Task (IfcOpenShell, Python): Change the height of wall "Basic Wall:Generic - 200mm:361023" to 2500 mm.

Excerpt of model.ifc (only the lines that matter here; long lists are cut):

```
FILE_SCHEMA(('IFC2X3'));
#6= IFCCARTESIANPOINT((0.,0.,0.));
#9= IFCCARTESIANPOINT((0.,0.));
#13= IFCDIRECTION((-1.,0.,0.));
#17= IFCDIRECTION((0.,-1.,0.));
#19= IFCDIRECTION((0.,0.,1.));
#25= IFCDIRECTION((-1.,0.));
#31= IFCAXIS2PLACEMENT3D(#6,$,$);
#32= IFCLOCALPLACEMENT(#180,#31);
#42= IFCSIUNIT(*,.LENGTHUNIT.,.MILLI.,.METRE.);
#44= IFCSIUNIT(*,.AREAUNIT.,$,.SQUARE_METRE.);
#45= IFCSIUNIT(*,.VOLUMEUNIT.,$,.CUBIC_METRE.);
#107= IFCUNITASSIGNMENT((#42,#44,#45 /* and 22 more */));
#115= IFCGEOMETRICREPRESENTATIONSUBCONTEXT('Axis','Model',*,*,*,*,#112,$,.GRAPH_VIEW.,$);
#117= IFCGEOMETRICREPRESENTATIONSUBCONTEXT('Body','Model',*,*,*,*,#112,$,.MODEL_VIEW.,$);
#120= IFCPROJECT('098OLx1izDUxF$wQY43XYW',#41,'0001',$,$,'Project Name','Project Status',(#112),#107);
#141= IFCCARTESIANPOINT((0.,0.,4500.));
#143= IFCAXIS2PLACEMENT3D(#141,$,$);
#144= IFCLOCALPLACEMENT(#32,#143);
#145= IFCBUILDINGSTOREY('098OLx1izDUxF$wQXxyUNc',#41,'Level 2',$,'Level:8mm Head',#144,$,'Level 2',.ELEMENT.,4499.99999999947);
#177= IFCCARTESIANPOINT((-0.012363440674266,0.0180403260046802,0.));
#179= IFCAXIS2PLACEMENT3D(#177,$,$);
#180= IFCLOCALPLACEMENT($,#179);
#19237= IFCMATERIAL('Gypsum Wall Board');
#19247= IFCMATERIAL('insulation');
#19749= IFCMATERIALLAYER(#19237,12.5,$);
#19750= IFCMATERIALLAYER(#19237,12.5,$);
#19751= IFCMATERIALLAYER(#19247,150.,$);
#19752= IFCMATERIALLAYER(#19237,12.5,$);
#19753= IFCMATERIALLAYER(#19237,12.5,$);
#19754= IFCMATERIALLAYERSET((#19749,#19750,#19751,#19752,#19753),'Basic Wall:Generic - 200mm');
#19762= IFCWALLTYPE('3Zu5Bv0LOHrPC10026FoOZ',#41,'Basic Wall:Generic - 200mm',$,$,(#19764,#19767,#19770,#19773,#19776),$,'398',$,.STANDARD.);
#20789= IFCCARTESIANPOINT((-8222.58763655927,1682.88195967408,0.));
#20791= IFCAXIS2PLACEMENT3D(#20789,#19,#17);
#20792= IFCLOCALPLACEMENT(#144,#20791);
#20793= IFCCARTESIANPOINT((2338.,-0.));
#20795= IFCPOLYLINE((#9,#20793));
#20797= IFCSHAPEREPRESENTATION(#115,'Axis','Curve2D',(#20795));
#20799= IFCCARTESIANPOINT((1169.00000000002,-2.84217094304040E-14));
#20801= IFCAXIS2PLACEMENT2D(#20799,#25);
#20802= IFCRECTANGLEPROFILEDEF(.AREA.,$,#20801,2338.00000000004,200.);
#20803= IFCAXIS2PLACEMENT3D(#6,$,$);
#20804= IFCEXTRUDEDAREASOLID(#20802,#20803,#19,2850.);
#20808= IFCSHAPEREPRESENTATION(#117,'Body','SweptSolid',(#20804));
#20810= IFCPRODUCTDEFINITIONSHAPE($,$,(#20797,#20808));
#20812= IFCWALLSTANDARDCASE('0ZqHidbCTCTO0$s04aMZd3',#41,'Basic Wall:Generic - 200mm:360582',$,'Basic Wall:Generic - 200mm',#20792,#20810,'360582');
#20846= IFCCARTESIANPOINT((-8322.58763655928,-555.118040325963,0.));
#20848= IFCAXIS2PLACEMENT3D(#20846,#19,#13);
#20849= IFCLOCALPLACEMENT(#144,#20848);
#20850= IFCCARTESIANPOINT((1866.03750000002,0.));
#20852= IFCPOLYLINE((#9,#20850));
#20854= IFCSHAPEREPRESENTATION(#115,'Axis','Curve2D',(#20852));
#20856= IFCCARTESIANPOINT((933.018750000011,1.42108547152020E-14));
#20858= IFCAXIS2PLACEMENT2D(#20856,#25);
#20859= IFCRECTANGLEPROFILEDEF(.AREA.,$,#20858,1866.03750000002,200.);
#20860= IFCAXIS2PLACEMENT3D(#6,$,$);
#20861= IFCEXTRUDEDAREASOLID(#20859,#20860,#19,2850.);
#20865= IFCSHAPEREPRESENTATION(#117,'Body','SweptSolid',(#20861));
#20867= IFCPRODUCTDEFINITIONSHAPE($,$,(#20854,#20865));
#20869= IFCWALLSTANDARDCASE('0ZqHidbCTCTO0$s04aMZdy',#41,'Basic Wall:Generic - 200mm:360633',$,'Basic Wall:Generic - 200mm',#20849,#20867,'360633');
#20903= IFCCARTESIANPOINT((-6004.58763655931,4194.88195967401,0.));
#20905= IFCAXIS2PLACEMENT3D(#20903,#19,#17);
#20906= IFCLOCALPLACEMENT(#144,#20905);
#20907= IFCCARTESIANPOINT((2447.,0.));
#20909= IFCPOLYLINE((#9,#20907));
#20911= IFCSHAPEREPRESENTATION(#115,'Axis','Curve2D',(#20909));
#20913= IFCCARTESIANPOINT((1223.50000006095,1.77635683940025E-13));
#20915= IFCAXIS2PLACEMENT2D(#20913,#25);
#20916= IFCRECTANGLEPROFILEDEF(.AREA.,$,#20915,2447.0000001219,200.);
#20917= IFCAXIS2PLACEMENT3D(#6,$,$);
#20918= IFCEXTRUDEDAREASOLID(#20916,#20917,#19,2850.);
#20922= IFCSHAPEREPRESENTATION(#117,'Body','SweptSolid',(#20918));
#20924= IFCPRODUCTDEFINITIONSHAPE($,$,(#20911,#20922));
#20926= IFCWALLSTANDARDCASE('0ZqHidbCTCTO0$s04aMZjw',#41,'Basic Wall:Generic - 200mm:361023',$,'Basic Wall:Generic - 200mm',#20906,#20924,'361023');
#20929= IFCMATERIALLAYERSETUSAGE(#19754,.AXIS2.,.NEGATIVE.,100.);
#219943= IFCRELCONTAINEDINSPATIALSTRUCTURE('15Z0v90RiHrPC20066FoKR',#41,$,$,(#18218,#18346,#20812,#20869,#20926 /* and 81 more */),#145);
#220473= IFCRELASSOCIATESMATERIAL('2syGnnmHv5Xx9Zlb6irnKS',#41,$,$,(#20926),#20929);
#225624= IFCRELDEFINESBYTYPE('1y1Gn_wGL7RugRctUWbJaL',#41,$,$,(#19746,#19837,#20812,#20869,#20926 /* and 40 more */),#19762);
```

```python
import ifcopenshell
import ifcopenshell.geom
import ifcopenshell.util.representation
import ifcopenshell.util.shape
import ifcopenshell.util.unit

model = ifcopenshell.open("model.ifc")
unit_scale = ifcopenshell.util.unit.calculate_unit_scale(model)
settings = ifcopenshell.geom.settings()


def volume(element):
    """Net volume in cubic metres, openings subtracted."""
    shape = ifcopenshell.geom.create_shape(settings, element)
    return ifcopenshell.util.shape.get_volume(shape.geometry)


wall = model.by_guid("0ZqHidbCTCTO0$s04aMZjw")
before = volume(wall)

body = ifcopenshell.util.representation.get_representation(wall, "Model", "Body")
solid = body.Items[0]
old_height = solid.Depth
solid.Depth = 2.5 / unit_scale
after = volume(wall)

print(f"height {old_height:g} -> {solid.Depth:g}, volume {before:.3f} -> {after:.3f} m3")

model.write("model_rev.ifc")
```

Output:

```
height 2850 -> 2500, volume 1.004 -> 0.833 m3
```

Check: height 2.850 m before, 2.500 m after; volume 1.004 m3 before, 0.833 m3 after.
